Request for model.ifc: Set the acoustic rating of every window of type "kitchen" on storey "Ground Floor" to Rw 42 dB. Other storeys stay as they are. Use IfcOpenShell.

First a look at what the model holds.

```python
import ifcopenshell
import ifcopenshell.util.element

model = ifcopenshell.open("model.ifc")
print(model.schema)
storey = next(s for s in model.by_type("IfcBuildingStorey") if s.Name == "Ground Floor")
windows = [e for e in ifcopenshell.util.element.get_decomposition(storey) if e.is_a("IfcWindow")]
seen = {}
for e in windows:
    element_type = ifcopenshell.util.element.get_type(e)
    key = (element_type.Name if element_type != e and element_type else None, ifcopenshell.util.element.get_pset(e, "Pset_WindowCommon", "AcousticRating"))
    seen[key] = seen.get(key, 0) + 1
for (name, value), count in sorted(seen.items(), key=str):
    print(count, "x", name, "|", value)
```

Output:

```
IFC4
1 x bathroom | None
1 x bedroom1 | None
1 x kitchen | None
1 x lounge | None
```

```python
import ifcopenshell
import ifcopenshell.api.pset
import ifcopenshell.util.element

model = ifcopenshell.open("model.ifc")

storey = next(s for s in model.by_type("IfcBuildingStorey") if s.Name == "Ground Floor")
windows = [e for e in ifcopenshell.util.element.get_decomposition(storey) if e.is_a("IfcWindow")]

count = 0
for e in windows:
    element_type = ifcopenshell.util.element.get_type(e)
    if element_type in (None, e) or element_type.Name != "kitchen":
        continue
    # add_pset returns the element's existing set when there is one.
    pset = ifcopenshell.api.pset.add_pset(model, product=e, name="Pset_WindowCommon")
    ifcopenshell.api.pset.edit_pset(model, pset=pset, properties={"AcousticRating": "Rw 42 dB"})
    count += 1

print(count, "windows updated")

model.write("model_rev.ifc")
```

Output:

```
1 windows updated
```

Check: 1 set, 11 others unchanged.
